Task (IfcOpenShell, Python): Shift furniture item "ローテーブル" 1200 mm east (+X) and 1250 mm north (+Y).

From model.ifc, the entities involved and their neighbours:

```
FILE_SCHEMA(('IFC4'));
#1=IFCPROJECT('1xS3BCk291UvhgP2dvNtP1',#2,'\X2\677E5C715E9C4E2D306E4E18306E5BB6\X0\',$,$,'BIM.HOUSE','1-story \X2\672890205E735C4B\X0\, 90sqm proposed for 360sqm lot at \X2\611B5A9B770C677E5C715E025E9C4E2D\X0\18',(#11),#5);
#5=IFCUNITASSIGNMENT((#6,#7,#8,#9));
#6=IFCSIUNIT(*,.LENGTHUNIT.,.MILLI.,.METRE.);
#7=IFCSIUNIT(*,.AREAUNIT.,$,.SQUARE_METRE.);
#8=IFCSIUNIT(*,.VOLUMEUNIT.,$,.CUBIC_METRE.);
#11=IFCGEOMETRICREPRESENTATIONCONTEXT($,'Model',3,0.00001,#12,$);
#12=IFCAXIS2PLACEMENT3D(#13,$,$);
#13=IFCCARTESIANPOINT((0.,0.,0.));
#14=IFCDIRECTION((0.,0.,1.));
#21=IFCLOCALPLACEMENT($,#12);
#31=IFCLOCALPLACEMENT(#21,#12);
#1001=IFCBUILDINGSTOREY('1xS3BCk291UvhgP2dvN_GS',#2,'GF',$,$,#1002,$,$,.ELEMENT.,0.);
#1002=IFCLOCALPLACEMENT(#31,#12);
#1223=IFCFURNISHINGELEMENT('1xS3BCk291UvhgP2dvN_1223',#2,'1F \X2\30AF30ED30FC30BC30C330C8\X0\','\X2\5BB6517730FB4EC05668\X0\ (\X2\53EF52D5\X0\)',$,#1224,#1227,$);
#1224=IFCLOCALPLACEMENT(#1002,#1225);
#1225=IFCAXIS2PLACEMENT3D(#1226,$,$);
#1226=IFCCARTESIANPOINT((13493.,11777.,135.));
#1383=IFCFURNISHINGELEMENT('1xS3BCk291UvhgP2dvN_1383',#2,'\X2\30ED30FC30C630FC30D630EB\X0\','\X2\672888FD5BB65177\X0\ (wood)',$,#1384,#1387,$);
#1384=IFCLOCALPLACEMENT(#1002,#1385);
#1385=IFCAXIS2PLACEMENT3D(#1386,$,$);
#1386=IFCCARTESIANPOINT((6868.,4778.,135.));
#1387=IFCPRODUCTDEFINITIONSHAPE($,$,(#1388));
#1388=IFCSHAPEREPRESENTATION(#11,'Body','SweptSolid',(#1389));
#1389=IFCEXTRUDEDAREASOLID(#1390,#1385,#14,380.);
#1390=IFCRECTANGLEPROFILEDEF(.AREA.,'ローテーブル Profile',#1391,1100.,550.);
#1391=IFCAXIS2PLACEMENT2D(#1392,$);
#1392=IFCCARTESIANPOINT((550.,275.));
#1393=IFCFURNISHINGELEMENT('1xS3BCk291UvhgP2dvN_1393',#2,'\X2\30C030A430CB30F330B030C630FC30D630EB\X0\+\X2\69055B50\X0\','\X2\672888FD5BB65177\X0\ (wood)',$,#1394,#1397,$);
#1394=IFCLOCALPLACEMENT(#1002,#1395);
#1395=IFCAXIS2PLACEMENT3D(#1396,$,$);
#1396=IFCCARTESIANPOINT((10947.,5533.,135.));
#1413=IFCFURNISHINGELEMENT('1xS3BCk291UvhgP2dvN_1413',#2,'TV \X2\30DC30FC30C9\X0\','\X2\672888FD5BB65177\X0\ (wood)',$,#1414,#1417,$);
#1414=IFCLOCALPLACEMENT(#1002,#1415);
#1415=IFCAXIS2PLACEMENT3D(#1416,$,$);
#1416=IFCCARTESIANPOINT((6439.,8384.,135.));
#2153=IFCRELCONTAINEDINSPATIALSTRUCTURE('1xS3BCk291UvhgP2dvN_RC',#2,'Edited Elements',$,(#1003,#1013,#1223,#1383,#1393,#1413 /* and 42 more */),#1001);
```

```python
import ifcopenshell
import ifcopenshell.api.geometry
import ifcopenshell.util.placement

model = ifcopenshell.open("model.ifc")

item = model.by_id(1383)
matrix = ifcopenshell.util.placement.get_local_placement(item.ObjectPlacement)
matrix[0, 3] += 1200.0
matrix[1, 3] += 1250.0
ifcopenshell.api.geometry.edit_object_placement(model, product=item, matrix=matrix, is_si=False)

print(ifcopenshell.util.placement.get_local_placement(item.ObjectPlacement).round(3) + 0.0)

model.write("model_updated.ifc")
```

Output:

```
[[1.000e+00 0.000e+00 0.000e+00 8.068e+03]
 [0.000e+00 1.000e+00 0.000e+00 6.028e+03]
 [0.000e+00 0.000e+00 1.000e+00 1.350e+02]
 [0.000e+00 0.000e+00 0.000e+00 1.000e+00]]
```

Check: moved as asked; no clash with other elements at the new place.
